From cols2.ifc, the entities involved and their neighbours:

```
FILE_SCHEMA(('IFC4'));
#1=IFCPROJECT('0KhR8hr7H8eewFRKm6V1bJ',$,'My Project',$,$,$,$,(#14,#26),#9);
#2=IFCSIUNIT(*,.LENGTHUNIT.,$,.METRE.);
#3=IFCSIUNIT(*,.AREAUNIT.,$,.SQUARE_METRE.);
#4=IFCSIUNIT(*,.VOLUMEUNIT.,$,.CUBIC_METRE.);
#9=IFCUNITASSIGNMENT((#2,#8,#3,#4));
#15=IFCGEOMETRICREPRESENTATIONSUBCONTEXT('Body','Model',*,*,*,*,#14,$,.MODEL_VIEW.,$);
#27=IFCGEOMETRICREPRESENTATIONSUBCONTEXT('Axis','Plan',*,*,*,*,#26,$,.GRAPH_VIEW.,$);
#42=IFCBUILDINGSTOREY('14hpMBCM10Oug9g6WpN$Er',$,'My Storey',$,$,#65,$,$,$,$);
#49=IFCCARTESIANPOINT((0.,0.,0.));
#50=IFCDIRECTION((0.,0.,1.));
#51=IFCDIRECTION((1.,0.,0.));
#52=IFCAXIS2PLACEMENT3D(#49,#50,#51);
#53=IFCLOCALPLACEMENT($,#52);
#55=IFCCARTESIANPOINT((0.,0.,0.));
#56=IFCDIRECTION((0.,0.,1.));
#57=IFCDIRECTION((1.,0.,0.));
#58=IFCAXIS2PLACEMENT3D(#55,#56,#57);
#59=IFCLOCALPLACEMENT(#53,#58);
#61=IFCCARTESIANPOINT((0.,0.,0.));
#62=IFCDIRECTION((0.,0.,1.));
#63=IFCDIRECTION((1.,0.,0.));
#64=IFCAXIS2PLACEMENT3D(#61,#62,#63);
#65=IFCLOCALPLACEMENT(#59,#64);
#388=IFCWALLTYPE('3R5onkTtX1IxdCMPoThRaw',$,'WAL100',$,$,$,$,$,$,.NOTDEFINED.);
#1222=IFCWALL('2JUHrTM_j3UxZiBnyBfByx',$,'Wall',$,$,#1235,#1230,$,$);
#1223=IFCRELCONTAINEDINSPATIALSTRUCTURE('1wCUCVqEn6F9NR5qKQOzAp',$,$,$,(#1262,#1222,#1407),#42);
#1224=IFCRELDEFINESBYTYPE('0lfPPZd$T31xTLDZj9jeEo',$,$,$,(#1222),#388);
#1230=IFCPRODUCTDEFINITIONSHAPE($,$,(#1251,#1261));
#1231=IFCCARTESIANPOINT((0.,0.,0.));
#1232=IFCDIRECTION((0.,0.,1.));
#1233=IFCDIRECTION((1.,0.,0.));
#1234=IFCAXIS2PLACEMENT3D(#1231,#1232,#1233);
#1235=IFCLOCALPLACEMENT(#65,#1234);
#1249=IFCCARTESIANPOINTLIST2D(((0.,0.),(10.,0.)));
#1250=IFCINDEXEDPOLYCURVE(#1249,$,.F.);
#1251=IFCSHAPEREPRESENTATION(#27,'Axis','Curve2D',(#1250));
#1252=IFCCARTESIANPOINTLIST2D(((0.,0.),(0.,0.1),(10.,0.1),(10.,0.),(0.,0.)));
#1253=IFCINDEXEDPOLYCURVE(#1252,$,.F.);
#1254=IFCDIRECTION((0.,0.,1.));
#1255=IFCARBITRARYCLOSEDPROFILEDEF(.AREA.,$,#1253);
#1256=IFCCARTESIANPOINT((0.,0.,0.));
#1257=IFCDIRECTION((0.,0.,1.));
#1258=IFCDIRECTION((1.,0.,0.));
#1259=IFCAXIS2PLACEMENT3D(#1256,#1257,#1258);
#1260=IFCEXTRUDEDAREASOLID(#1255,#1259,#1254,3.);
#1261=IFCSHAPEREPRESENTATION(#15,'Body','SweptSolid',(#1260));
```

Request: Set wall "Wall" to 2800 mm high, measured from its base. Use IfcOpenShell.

```python
import ifcopenshell
import ifcopenshell.geom
import ifcopenshell.util.representation
import ifcopenshell.util.shape
import ifcopenshell.util.unit

model = ifcopenshell.open("cols2.ifc")
unit_scale = ifcopenshell.util.unit.calculate_unit_scale(model)
settings = ifcopenshell.geom.settings()


def volume(element):
    """Net volume in cubic metres, openings subtracted."""
    shape = ifcopenshell.geom.create_shape(settings, element)
    return ifcopenshell.util.shape.get_volume(shape.geometry)


wall = model.by_guid("2JUHrTM_j3UxZiBnyBfByx")
before = volume(wall)

body = ifcopenshell.util.representation.get_representation(wall, "Model", "Body")
solid = body.Items[0]
old_height = solid.Depth
solid.Depth = 2.8 / unit_scale
after = volume(wall)

print(f"height {old_height:g} -> {solid.Depth:g}, volume {before:.3f} -> {after:.3f} m3")

model.write("cols2_edited.ifc")
```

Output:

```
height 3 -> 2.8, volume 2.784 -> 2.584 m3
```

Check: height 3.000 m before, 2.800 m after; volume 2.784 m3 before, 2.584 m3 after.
